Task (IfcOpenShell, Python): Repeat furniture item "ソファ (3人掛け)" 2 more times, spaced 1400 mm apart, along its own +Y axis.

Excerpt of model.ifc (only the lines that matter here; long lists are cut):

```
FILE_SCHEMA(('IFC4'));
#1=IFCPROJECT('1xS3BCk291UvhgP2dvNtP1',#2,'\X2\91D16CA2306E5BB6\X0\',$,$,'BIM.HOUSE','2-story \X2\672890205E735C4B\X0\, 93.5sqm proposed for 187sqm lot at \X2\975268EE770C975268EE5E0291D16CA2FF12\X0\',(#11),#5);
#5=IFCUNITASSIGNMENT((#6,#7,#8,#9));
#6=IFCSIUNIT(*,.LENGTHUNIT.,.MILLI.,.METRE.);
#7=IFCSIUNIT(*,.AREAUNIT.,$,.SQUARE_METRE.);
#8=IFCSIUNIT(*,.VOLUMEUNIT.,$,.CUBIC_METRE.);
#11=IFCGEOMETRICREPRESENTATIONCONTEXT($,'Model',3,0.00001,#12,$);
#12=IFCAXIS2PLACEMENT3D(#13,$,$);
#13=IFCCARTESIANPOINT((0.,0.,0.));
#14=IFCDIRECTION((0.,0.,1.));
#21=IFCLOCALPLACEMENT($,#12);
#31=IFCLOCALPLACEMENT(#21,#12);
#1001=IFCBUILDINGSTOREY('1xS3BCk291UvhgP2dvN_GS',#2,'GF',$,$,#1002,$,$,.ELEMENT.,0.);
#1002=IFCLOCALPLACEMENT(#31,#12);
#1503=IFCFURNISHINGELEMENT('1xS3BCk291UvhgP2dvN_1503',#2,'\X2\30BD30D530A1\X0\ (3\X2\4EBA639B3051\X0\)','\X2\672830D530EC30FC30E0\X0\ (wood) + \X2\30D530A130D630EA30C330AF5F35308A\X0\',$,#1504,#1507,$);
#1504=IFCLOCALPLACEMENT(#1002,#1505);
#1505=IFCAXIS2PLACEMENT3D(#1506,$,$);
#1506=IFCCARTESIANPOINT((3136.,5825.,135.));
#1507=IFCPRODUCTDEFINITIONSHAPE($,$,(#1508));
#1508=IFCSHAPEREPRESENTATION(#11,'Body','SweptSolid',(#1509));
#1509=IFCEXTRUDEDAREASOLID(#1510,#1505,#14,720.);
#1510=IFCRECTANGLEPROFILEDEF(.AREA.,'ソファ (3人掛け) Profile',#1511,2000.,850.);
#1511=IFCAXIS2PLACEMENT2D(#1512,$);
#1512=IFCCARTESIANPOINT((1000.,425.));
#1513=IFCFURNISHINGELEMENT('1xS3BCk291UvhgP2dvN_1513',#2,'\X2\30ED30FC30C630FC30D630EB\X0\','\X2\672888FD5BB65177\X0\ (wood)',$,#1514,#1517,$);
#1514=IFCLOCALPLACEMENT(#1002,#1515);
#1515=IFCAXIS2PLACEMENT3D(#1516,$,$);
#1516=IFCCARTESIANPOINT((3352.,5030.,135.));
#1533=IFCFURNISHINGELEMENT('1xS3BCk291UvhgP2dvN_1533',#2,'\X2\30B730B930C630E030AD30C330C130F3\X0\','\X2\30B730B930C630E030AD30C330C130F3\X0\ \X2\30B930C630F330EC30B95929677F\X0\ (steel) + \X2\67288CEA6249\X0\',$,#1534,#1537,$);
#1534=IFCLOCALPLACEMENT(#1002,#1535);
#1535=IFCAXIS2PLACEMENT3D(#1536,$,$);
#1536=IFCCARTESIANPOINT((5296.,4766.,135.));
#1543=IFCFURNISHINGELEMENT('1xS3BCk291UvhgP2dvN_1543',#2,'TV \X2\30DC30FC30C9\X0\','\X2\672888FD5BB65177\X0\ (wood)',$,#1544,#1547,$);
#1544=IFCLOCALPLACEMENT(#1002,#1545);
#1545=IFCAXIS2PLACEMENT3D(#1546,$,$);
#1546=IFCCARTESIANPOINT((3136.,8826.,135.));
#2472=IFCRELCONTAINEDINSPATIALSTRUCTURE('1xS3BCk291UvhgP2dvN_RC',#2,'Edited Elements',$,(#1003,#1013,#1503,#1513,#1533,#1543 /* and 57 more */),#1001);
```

```python
import ifcopenshell
import ifcopenshell.api.geometry
import ifcopenshell.api.root
import ifcopenshell.util.element
import ifcopenshell.util.placement
import ifcopenshell.util.unit

model = ifcopenshell.open("model.ifc")
unit_scale = ifcopenshell.util.unit.calculate_unit_scale(model)


def reuse_history(source, copy):
    """copy_class also copies each property set's owner history, people and application; keep the originals."""
    for rel in copy.IsDefinedBy:
        if rel.is_a("IfcRelDefinesByProperties") and (history := rel.RelatingPropertyDefinition.OwnerHistory):
            rel.RelatingPropertyDefinition.OwnerHistory = source.OwnerHistory
            ifcopenshell.util.element.remove_deep2(model, history)


source = model.by_guid("1xS3BCk291UvhgP2dvN_1503")
base = ifcopenshell.util.placement.get_local_placement(source.ObjectPlacement)
step = base[:3, 1] * 1.4 / unit_scale

for i in range(1, 3):
    copy = ifcopenshell.api.root.copy_class(model, product=source)
    copy.Representation = ifcopenshell.util.element.copy_deep(
        model, source.Representation, exclude=["IfcGeometricRepresentationContext", "IfcRepresentationMap"]
    )
    reuse_history(source, copy)
    matrix = base.copy()
    matrix[:3, 3] += i * step
    print("added at", matrix[:3, 3].round(3) + 0.0)
    ifcopenshell.api.geometry.edit_object_placement(model, product=copy, matrix=matrix, is_si=False)

model.write("model_v2.ifc")
```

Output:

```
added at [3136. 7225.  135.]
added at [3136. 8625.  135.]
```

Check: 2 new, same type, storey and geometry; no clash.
